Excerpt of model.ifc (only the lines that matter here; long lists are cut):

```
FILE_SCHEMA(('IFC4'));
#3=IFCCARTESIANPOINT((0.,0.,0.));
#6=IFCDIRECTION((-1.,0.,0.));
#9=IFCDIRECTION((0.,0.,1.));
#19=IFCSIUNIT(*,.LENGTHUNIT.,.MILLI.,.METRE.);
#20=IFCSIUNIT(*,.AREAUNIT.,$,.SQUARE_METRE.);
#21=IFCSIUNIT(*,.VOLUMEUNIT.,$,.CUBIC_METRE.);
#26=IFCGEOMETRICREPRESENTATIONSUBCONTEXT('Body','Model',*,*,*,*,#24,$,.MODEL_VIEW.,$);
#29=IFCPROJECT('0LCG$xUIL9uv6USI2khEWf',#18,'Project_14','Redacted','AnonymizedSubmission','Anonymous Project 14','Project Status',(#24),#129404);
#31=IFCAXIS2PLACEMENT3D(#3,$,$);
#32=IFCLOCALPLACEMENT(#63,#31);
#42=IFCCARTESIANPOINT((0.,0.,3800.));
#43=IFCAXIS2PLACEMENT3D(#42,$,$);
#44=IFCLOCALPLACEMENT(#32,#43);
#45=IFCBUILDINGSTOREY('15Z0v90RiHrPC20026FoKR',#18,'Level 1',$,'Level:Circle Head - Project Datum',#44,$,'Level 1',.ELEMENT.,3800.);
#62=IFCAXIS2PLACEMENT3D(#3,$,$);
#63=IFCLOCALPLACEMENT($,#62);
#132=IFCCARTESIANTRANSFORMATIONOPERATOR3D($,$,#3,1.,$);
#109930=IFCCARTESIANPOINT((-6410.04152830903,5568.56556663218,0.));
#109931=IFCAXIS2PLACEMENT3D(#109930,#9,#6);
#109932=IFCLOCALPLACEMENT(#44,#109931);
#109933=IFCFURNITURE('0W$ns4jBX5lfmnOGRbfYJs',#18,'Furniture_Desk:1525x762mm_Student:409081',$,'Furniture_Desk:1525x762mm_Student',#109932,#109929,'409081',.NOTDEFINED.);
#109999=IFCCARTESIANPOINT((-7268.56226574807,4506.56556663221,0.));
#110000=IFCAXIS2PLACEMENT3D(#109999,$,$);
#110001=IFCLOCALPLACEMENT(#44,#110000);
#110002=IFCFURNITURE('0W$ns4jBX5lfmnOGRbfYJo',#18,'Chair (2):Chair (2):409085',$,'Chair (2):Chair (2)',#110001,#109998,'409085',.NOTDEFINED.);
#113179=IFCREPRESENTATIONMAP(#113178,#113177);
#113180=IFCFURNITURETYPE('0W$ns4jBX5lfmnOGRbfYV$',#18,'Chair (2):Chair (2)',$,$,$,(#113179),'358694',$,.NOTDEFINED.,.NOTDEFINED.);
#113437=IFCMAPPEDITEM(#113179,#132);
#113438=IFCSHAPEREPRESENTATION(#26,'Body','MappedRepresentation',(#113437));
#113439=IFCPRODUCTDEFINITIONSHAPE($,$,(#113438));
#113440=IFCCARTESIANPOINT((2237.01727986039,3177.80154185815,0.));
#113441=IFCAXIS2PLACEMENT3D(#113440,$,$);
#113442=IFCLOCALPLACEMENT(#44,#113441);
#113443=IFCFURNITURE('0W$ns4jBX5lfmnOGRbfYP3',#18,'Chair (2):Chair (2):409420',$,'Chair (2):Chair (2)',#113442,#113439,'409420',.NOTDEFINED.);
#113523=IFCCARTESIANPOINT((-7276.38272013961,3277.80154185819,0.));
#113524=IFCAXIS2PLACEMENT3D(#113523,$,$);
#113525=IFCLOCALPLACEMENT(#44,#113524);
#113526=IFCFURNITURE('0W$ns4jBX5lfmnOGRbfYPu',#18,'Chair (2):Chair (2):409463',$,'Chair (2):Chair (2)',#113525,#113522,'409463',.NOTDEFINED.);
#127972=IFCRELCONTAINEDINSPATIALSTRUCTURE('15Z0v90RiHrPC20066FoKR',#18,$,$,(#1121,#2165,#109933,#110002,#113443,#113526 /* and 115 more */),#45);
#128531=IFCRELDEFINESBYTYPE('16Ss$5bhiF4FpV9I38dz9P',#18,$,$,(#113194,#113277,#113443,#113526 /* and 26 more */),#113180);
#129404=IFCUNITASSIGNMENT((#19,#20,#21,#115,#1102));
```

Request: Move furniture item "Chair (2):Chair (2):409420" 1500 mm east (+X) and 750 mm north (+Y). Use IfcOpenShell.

```python
import ifcopenshell
import ifcopenshell.api.geometry
import ifcopenshell.util.placement
import ifcopenshell.util.unit

model = ifcopenshell.open("model.ifc")
unit_scale = ifcopenshell.util.unit.calculate_unit_scale(model)

item = model.by_guid("0W$ns4jBX5lfmnOGRbfYP3")
matrix = ifcopenshell.util.placement.get_local_placement(item.ObjectPlacement)
matrix[0, 3] += 1.5 / unit_scale
matrix[1, 3] += 0.75 / unit_scale
ifcopenshell.api.geometry.edit_object_placement(model, product=item, matrix=matrix, is_si=False)

print(ifcopenshell.util.placement.get_local_placement(item.ObjectPlacement).round(3) + 0.0)

model.write("model_updated.ifc")
```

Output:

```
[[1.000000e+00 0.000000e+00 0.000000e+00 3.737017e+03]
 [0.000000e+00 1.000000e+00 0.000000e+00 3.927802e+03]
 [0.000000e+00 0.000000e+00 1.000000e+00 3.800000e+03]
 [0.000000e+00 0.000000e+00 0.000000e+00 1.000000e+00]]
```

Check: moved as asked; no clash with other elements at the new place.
